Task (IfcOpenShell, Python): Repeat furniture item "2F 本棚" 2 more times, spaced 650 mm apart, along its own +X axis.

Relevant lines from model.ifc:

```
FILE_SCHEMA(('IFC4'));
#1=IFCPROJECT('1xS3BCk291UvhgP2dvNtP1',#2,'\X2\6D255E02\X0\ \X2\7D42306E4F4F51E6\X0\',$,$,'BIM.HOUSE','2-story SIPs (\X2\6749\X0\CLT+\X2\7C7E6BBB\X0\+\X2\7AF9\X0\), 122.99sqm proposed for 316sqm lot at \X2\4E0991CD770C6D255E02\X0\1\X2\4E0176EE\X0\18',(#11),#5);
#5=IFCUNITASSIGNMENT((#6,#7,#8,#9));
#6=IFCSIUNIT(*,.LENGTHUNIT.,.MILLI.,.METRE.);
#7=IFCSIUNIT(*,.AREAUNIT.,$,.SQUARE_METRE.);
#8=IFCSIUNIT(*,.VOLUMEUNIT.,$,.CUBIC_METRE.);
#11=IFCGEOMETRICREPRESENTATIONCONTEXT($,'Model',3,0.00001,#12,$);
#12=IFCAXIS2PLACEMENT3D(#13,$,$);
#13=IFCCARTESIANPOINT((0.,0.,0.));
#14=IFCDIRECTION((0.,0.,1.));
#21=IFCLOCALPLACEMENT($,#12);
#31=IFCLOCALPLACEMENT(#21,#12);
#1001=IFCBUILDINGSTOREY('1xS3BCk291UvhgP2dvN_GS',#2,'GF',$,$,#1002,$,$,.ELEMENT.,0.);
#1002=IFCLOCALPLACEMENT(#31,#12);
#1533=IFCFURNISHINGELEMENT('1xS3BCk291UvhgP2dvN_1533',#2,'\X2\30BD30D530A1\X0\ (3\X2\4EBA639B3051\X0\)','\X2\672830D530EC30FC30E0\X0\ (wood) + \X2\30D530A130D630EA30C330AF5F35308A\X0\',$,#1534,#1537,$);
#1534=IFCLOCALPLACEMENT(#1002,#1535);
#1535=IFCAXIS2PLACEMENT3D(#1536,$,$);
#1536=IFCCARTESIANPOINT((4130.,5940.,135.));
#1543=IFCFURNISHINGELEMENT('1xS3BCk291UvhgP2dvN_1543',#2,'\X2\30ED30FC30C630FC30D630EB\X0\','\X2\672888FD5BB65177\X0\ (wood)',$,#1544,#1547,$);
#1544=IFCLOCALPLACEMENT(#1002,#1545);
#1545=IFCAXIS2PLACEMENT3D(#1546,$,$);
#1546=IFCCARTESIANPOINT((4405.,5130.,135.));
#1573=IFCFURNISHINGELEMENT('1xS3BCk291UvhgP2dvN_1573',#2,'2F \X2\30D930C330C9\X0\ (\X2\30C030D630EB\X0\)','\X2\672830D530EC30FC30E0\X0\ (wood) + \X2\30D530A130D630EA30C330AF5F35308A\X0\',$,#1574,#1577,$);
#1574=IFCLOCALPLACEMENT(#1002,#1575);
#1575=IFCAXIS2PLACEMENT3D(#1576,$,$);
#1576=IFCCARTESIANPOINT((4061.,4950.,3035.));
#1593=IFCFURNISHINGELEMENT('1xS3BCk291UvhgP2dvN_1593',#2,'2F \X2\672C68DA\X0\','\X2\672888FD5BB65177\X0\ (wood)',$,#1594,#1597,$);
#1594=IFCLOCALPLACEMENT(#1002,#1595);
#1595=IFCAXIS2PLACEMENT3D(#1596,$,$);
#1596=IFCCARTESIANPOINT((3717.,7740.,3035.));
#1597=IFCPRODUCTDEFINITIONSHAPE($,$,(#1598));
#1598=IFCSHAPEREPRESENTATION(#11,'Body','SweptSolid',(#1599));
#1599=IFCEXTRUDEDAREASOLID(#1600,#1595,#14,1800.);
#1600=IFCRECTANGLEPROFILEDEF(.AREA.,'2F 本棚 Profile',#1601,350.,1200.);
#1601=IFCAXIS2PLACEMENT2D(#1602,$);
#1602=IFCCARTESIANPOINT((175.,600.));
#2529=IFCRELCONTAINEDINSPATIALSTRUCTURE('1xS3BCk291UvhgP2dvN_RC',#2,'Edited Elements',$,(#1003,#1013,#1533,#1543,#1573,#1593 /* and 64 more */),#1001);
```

```python
import ifcopenshell
import ifcopenshell.api.geometry
import ifcopenshell.api.root
import ifcopenshell.util.element
import ifcopenshell.util.placement
import ifcopenshell.util.unit

model = ifcopenshell.open("model.ifc")
unit_scale = ifcopenshell.util.unit.calculate_unit_scale(model)


def reuse_history(source, copy):
    """copy_class also copies each property set's owner history, people and application; keep the originals."""
    for rel in copy.IsDefinedBy:
        if rel.is_a("IfcRelDefinesByProperties") and (history := rel.RelatingPropertyDefinition.OwnerHistory):
            rel.RelatingPropertyDefinition.OwnerHistory = source.OwnerHistory
            ifcopenshell.util.element.remove_deep2(model, history)


source = model.by_guid("1xS3BCk291UvhgP2dvN_1593")
base = ifcopenshell.util.placement.get_local_placement(source.ObjectPlacement)
step = base[:3, 0] * 0.65 / unit_scale

for i in range(1, 3):
    copy = ifcopenshell.api.root.copy_class(model, product=source)
    copy.Representation = ifcopenshell.util.element.copy_deep(
        model, source.Representation, exclude=["IfcGeometricRepresentationContext", "IfcRepresentationMap"]
    )
    reuse_history(source, copy)
    matrix = base.copy()
    matrix[:3, 3] += i * step
    print("added at", matrix[:3, 3].round(3) + 0.0)
    ifcopenshell.api.geometry.edit_object_placement(model, product=copy, matrix=matrix, is_si=False)

model.write("model-out.ifc")
```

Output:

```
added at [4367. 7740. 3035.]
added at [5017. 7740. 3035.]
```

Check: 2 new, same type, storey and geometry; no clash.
